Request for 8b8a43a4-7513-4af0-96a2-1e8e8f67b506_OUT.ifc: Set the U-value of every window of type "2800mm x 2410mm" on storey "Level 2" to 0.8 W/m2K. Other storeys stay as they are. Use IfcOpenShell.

First a look at what the model holds.

```python
import ifcopenshell
import ifcopenshell.util.element

model = ifcopenshell.open("8b8a43a4-7513-4af0-96a2-1e8e8f67b506_OUT.ifc")
print(model.schema)
storey = next(s for s in model.by_type("IfcBuildingStorey") if s.Name == "Level 2")
windows = [e for e in ifcopenshell.util.element.get_decomposition(storey) if e.is_a("IfcWindow")]
seen = {}
for e in windows:
    element_type = ifcopenshell.util.element.get_type(e)
    key = (element_type.Name if element_type != e and element_type else None, ifcopenshell.util.element.get_pset(e, "Pset_WindowCommon", "ThermalTransmittance"))
    seen[key] = seen.get(key, 0) + 1
for (name, value), count in sorted(seen.items(), key=str):
    print(count, "x", name, "|", value)
```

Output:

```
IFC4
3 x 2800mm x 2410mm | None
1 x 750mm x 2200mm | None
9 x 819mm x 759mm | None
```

```python
import ifcopenshell
import ifcopenshell.api.pset
import ifcopenshell.util.element

model = ifcopenshell.open("8b8a43a4-7513-4af0-96a2-1e8e8f67b506_OUT.ifc")

storey = next(s for s in model.by_type("IfcBuildingStorey") if s.Name == "Level 2")
windows = [e for e in ifcopenshell.util.element.get_decomposition(storey) if e.is_a("IfcWindow")]

count = 0
for e in windows:
    element_type = ifcopenshell.util.element.get_type(e)
    if element_type in (None, e) or element_type.Name != "2800mm x 2410mm":
        continue
    # add_pset returns the element's existing set when there is one.
    pset = ifcopenshell.api.pset.add_pset(model, product=e, name="Pset_WindowCommon")
    ifcopenshell.api.pset.edit_pset(model, pset=pset, properties={"ThermalTransmittance": 0.8})
    count += 1

print(count, "windows updated")

model.write("8b8a43a4-7513-4af0-96a2-1e8e8f67b506_OUT_rev.ifc")
```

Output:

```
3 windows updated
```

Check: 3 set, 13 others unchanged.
